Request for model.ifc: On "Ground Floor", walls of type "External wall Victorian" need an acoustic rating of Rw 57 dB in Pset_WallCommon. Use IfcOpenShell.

First a look at what the model holds.

```python
import ifcopenshell
import ifcopenshell.util.element

model = ifcopenshell.open("model.ifc")
print(model.schema)
storey = next(s for s in model.by_type("IfcBuildingStorey") if s.Name == "Ground Floor")
walls = [e for e in ifcopenshell.util.element.get_decomposition(storey) if e.is_a("IfcWall")]
seen = {}
for e in walls:
    element_type = ifcopenshell.util.element.get_type(e)
    key = (element_type.Name if element_type != e and element_type else None, ifcopenshell.util.element.get_pset(e, "Pset_WallCommon", "AcousticRating"))
    seen[key] = seen.get(key, 0) + 1
for (name, value), count in sorted(seen.items(), key=str):
    print(count, "x", name, "|", value)
```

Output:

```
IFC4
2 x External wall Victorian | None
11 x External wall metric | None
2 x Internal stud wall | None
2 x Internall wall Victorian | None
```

```python
import ifcopenshell
import ifcopenshell.api.pset
import ifcopenshell.util.element

model = ifcopenshell.open("model.ifc")

storey = next(s for s in model.by_type("IfcBuildingStorey") if s.Name == "Ground Floor")
walls = [e for e in ifcopenshell.util.element.get_decomposition(storey) if e.is_a("IfcWall")]

count = 0
for e in walls:
    element_type = ifcopenshell.util.element.get_type(e)
    if element_type in (None, e) or element_type.Name != "External wall Victorian":
        continue
    # add_pset returns the element's existing set when there is one.
    pset = ifcopenshell.api.pset.add_pset(model, product=e, name="Pset_WallCommon")
    ifcopenshell.api.pset.edit_pset(model, pset=pset, properties={"AcousticRating": "Rw 57 dB"})
    count += 1

print(count, "walls updated")

model.write("model_edited.ifc")
```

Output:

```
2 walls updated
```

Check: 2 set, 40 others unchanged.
